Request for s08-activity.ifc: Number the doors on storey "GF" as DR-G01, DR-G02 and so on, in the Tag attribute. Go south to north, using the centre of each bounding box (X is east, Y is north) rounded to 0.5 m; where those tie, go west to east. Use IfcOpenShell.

First a look at what the model holds.

```python
import ifcopenshell
import ifcopenshell.util.element
import ifcopenshell.util.placement

model = ifcopenshell.open("s08-activity.ifc")
print(model.schema)
storey = next(s for s in model.by_type("IfcBuildingStorey") if s.Name == "GF")
doors = [e for e in ifcopenshell.util.element.get_decomposition(storey) if e.is_a("IfcDoor")]
for e in sorted(doors, key=lambda e: e.id()):
    origin = ifcopenshell.util.placement.get_local_placement(e.ObjectPlacement)[:3, 3]
    print(e.id(), e.Tag, e.Name, origin.round(2) + 0.0, sep=" | ")
```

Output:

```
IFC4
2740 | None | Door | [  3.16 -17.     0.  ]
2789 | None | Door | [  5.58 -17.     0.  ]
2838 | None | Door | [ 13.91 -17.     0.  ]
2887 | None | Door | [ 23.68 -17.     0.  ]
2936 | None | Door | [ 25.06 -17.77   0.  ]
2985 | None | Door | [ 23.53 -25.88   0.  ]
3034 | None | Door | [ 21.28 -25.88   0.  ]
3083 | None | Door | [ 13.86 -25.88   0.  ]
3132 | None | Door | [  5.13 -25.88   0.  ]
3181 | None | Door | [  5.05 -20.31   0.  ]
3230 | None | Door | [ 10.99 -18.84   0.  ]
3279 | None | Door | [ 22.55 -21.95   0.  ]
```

```python
import ifcopenshell
import ifcopenshell.geom
import ifcopenshell.util.element
import ifcopenshell.util.shape

model = ifcopenshell.open("s08-activity.ifc")
settings = ifcopenshell.geom.settings()
settings.set("use-world-coords", True)


def centre(element):
    shape = ifcopenshell.geom.create_shape(settings, element)
    return ifcopenshell.util.shape.get_bbox_centroid(shape.geometry)


storey = next(s for s in model.by_type("IfcBuildingStorey") if s.Name == "GF")
doors = [e for e in ifcopenshell.util.element.get_decomposition(storey) if e.is_a("IfcDoor")]

# Insertion points can sit at a corner or the storey origin, so sort by the geometry (in metres).
centres = {e: centre(e) for e in doors}
doors.sort(key=lambda e: (round(centres[e][1] / 0.5), centres[e][0]))

for i, e in enumerate(doors, start=1):
    number = f"DR-G{i:02d}"
    e.Tag = number
    print(e.id(), number)

model.write("s08-activity_rev.ifc")
```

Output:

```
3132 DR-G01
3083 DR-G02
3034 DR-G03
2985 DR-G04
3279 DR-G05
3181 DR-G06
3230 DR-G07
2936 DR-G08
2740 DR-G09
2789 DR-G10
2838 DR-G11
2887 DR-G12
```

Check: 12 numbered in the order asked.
